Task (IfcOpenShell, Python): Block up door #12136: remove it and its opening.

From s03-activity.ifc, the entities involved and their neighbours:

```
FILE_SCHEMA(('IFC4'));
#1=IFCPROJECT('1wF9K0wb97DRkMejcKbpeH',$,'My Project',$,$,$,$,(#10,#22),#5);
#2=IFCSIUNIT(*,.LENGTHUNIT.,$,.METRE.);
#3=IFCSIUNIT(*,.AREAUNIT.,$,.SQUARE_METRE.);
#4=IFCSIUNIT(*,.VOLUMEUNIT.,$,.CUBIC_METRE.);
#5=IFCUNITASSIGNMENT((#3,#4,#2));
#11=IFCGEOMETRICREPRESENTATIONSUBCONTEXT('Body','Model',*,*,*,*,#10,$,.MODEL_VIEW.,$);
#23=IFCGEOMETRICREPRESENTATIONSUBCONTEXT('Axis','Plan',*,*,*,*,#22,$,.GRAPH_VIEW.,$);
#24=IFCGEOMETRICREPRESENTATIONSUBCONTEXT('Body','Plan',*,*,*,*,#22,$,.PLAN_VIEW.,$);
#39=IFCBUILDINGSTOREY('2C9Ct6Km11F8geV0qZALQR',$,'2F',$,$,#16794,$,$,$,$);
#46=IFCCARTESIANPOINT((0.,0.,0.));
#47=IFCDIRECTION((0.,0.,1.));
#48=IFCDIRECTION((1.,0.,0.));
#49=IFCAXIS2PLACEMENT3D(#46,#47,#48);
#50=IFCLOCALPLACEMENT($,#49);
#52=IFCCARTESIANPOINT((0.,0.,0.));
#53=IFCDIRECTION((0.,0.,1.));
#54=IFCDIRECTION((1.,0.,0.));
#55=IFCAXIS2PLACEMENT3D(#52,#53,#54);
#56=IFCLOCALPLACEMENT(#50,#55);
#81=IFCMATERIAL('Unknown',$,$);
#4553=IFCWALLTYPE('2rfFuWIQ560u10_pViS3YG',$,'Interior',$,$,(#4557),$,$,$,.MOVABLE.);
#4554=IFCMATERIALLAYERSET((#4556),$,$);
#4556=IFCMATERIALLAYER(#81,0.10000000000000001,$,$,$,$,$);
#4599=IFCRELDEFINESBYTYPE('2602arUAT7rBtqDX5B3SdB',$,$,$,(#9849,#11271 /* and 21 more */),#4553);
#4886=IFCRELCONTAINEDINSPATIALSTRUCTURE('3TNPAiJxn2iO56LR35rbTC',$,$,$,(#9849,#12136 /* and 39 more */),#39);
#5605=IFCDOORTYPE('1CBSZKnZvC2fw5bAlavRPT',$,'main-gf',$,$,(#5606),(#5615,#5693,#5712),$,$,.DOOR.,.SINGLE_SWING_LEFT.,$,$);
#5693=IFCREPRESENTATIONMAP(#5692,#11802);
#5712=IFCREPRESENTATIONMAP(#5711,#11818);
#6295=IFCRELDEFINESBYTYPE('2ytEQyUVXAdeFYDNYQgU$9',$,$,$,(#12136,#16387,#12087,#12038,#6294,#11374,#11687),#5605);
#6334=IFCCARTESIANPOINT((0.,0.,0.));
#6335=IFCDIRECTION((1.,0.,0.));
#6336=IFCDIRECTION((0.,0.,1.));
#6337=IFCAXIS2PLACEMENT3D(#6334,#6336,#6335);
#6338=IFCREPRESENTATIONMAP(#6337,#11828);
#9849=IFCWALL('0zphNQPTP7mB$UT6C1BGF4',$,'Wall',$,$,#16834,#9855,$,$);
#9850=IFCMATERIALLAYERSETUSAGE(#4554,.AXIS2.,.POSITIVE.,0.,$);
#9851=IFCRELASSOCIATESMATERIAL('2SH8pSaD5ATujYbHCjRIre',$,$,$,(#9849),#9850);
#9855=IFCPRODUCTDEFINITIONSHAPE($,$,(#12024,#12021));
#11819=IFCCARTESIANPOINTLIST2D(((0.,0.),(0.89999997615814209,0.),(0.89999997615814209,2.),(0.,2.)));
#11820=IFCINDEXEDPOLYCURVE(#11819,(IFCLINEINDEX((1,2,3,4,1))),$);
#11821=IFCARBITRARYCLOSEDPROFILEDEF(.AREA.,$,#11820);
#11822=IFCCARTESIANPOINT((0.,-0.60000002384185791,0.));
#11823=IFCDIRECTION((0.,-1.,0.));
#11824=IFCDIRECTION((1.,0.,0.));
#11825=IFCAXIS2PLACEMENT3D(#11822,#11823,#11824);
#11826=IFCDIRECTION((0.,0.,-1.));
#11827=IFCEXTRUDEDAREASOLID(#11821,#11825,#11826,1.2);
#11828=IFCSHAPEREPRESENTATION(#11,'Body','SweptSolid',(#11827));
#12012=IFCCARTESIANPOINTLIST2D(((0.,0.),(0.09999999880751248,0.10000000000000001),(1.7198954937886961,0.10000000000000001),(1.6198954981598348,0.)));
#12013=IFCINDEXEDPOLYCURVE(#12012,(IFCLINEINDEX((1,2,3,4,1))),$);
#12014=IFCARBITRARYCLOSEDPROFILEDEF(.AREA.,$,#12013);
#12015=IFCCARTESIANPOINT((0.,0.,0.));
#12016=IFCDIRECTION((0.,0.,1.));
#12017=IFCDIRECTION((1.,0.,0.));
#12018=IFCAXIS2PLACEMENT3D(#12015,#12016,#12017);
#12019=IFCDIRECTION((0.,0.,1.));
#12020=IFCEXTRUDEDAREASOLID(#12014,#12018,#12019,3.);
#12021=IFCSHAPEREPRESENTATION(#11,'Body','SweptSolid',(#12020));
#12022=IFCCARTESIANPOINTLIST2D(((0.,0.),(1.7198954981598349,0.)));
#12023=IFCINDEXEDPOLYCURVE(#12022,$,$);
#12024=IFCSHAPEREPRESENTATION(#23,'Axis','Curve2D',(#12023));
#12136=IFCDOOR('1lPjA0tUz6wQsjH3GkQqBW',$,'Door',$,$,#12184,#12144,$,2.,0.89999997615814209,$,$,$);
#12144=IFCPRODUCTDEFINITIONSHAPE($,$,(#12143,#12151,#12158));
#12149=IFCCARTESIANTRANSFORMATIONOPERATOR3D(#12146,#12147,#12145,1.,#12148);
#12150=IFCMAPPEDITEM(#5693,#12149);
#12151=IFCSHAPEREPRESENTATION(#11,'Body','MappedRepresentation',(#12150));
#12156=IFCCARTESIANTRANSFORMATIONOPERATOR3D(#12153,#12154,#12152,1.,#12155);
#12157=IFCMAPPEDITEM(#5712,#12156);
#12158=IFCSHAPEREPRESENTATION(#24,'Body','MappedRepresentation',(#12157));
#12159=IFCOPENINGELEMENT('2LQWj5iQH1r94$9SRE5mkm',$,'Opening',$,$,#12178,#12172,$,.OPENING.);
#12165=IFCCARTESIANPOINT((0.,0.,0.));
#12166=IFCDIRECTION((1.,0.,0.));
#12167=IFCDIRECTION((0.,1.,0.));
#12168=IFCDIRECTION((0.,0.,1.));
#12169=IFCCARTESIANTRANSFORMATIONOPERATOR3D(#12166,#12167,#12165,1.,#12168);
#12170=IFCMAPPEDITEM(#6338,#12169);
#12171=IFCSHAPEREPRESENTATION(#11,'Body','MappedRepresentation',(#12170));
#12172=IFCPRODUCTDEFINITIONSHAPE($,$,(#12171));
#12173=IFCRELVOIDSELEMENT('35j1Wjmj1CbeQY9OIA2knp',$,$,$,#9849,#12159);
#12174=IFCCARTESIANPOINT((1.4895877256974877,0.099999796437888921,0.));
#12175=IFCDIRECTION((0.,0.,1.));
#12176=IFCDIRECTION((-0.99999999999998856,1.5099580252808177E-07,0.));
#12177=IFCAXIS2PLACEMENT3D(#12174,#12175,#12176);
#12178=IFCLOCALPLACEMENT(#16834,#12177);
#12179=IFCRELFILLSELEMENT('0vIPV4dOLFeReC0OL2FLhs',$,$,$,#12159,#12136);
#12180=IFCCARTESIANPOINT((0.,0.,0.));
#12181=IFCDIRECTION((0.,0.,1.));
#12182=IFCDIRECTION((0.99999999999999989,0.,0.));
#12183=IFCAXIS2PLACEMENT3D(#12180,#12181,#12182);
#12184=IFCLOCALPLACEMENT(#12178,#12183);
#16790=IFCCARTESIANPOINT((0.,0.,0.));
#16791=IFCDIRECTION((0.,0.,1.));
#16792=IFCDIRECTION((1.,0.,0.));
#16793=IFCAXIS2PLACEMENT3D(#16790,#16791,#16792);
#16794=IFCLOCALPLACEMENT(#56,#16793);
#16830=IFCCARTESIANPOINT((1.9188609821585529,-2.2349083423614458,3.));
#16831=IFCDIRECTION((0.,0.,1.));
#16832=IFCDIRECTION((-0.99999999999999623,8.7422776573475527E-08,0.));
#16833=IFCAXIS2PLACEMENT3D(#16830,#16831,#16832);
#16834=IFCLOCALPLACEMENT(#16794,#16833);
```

```python
import ifcopenshell
import ifcopenshell.api.feature
import ifcopenshell.api.root
import ifcopenshell.geom
import ifcopenshell.util.shape

model = ifcopenshell.open("s03-activity.ifc")
settings = ifcopenshell.geom.settings()


def volume(element):
    """Net volume in cubic metres, openings subtracted."""
    shape = ifcopenshell.geom.create_shape(settings, element)
    return ifcopenshell.util.shape.get_volume(shape.geometry)


door = model.by_guid("1lPjA0tUz6wQsjH3GkQqBW")
opening = door.FillsVoids[0].RelatingOpeningElement
wall = opening.VoidsElements[0].RelatingBuildingElement
before = volume(wall)

ifcopenshell.api.root.remove_product(model, product=door)
ifcopenshell.api.feature.remove_feature(model, feature=opening)

after = volume(wall)

print(f"wall volume {before:.3f} -> {after:.3f} m3")

model.write("s03-activity-out.ifc")
```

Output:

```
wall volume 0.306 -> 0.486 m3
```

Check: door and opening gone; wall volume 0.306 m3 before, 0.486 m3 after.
